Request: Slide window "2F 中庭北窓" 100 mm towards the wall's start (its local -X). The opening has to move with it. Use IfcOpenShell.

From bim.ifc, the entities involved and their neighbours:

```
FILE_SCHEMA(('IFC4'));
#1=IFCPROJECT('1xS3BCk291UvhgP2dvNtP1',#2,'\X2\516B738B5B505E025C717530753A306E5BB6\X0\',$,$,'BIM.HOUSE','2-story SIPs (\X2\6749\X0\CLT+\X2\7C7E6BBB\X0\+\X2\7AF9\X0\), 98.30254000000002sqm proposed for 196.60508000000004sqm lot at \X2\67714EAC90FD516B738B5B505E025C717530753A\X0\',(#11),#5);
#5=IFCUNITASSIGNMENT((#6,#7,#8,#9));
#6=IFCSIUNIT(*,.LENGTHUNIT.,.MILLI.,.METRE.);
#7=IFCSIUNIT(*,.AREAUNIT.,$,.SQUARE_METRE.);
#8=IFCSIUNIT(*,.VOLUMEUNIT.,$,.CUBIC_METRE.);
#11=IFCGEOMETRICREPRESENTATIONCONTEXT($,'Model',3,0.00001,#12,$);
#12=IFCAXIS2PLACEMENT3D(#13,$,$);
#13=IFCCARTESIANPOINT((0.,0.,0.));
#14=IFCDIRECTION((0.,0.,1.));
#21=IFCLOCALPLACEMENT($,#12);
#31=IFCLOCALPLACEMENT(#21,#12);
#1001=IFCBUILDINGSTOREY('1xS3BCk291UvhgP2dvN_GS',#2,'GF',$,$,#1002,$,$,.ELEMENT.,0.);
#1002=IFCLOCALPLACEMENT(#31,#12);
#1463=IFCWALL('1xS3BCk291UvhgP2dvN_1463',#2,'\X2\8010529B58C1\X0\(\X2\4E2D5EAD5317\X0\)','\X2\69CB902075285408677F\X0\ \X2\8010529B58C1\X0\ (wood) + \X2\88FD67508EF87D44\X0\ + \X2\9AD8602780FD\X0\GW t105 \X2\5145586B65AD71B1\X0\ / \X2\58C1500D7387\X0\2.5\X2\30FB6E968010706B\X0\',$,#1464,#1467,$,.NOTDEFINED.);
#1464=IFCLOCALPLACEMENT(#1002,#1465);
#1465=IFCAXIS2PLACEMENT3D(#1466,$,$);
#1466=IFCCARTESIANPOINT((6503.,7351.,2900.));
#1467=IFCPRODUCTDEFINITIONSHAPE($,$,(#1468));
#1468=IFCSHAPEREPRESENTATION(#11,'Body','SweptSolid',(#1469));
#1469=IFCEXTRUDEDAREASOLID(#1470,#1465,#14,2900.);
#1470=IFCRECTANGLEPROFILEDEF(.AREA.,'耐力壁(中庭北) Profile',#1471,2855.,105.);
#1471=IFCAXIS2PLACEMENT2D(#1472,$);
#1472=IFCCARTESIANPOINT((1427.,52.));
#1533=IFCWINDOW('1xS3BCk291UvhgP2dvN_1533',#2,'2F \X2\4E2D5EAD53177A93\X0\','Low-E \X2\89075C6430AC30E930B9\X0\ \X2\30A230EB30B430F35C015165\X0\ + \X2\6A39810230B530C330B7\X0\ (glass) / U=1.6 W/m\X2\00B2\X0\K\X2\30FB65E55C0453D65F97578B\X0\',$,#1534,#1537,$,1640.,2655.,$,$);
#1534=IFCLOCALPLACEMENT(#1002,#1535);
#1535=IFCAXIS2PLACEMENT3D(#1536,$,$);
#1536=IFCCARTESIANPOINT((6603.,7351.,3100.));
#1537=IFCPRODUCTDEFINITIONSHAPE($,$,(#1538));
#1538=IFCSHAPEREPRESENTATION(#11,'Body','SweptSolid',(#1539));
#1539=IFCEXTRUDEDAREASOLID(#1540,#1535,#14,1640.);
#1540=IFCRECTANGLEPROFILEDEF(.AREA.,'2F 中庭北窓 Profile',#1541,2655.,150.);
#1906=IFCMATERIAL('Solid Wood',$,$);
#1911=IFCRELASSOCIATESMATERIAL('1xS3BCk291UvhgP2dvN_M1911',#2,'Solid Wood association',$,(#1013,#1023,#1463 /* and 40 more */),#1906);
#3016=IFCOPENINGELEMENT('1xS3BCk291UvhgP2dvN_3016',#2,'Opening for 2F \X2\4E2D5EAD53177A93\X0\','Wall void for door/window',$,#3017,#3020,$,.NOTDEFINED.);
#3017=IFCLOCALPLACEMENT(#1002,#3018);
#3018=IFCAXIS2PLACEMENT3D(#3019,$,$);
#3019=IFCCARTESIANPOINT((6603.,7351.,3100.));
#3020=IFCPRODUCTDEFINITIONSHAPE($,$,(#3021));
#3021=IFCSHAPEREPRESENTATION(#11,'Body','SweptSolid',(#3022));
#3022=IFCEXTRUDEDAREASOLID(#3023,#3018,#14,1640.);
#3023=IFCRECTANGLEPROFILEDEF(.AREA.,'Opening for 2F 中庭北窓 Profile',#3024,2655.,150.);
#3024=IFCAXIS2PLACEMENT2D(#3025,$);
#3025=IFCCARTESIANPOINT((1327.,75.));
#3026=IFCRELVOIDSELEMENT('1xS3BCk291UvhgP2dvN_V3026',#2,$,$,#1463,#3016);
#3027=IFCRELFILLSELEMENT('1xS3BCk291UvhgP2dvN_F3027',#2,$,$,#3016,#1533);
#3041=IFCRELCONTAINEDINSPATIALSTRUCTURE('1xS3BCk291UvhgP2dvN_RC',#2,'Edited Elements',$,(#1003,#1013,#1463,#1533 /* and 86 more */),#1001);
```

```python
import ifcopenshell
import ifcopenshell.api.geometry
import ifcopenshell.util.placement
import ifcopenshell.util.unit

model = ifcopenshell.open("bim.ifc")
unit_scale = ifcopenshell.util.unit.calculate_unit_scale(model)

window = model.by_id(1533)
opening = window.FillsVoids[0].RelatingOpeningElement
wall = opening.VoidsElements[0].RelatingBuildingElement

wall_matrix = ifcopenshell.util.placement.get_local_placement(wall.ObjectPlacement)
shift = wall_matrix[:3, 0] * -0.1 / unit_scale
before = ifcopenshell.util.placement.get_local_placement(window.ObjectPlacement)[:3, 3].copy()

# The window is not placed relative to its opening, so move both.
for product in (opening, window):
    matrix = ifcopenshell.util.placement.get_local_placement(product.ObjectPlacement)
    matrix[:3, 3] += shift
    ifcopenshell.api.geometry.edit_object_placement(model, product=product, matrix=matrix, is_si=False)

after = ifcopenshell.util.placement.get_local_placement(window.ObjectPlacement)[:3, 3]
print("window moved by", (after - before).round(3) + 0.0)

model.write("bim_rev.ifc")
```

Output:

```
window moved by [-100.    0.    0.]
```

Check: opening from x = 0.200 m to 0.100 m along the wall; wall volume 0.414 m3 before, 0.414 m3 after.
